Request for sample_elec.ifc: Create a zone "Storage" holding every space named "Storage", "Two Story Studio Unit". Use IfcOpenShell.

First a look at what the model holds.

```python
import ifcopenshell

model = ifcopenshell.open("sample_elec.ifc")
print(model.schema)
seen = {}
for space in model.by_type("IfcSpace"):
    seen[space.LongName] = seen.get(space.LongName, 0) + 1
for name, count in sorted(seen.items(), key=str):
    print(count, "x", name)
print("zones:", [z.Name for z in model.by_type("IfcZone")][:20])
```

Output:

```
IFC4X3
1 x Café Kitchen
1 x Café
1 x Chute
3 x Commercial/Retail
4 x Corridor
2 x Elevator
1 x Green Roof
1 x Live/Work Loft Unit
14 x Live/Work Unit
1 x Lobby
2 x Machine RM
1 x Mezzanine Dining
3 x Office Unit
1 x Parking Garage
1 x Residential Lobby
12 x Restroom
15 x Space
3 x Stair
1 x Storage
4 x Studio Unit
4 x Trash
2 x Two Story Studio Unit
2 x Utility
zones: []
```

```python
import ifcopenshell
import ifcopenshell.api.group
import ifcopenshell.api.root

model = ifcopenshell.open("sample_elec.ifc")

names = {"Storage", "Two Story Studio Unit"}
spaces = [s for s in model.by_type("IfcSpace") if s.LongName in names]

zone = ifcopenshell.api.root.create_entity(model, ifc_class="IfcZone", name="Storage")
ifcopenshell.api.group.assign_group(model, products=spaces, group=zone)
print(len(spaces), "spaces in", zone.Name)

model.write("sample_elec_updated.ifc")
```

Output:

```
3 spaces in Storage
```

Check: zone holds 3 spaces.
